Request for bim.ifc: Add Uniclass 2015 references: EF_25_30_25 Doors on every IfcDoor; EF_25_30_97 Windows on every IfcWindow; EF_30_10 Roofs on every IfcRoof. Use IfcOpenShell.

First a look at what the model holds.

```python
import ifcopenshell

model = ifcopenshell.open("bim.ifc")
print(model.schema)
print("classifications:", [c.Name for c in model.by_type("IfcClassification")])
for ifc_class in ("IfcDoor", "IfcRoof", "IfcStair", "IfcWall", "IfcWindow"):
    print(ifc_class, len(model.by_type(ifc_class)))
```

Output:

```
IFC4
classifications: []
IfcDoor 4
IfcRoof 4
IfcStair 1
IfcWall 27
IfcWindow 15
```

```python
import ifcopenshell
import ifcopenshell.api.classification

model = ifcopenshell.open("bim.ifc")

system = ifcopenshell.api.classification.add_classification(model, classification="Uniclass 2015")

codes = {
    "IfcDoor": ("EF_25_30_25", "Doors"),
    "IfcWindow": ("EF_25_30_97", "Windows"),
    "IfcRoof": ("EF_30_10", "Roofs"),
}
for ifc_class, (code, name) in codes.items():
    products = model.by_type(ifc_class)
    ifcopenshell.api.classification.add_reference(
        model, products=products, classification=system, identification=code, name=name
    )
    print(code, len(products))

model.write("bim_edited.ifc")
```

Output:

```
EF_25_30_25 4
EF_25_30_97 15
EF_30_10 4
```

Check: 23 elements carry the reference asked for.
